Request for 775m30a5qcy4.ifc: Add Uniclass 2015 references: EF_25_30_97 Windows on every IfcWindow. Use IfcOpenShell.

First a look at what the model holds.

```python
import ifcopenshell

model = ifcopenshell.open("775m30a5qcy4.ifc")
print(model.schema)
print("classifications:", [c.Name for c in model.by_type("IfcClassification")])
for ifc_class in ("IfcDoor", "IfcRoof", "IfcStair", "IfcWall", "IfcWindow"):
    print(ifc_class, len(model.by_type(ifc_class)))
```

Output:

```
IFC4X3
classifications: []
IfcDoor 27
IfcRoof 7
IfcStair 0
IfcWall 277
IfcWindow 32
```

```python
import ifcopenshell
import ifcopenshell.api.classification

model = ifcopenshell.open("775m30a5qcy4.ifc")

system = ifcopenshell.api.classification.add_classification(model, classification="Uniclass 2015")

codes = {
    "IfcWindow": ("EF_25_30_97", "Windows"),
}
for ifc_class, (code, name) in codes.items():
    products = model.by_type(ifc_class)
    ifcopenshell.api.classification.add_reference(
        model, products=products, classification=system, identification=code, name=name
    )
    print(code, len(products))

model.write("775m30a5qcy4_v2.ifc")
```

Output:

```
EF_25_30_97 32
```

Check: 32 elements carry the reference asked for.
